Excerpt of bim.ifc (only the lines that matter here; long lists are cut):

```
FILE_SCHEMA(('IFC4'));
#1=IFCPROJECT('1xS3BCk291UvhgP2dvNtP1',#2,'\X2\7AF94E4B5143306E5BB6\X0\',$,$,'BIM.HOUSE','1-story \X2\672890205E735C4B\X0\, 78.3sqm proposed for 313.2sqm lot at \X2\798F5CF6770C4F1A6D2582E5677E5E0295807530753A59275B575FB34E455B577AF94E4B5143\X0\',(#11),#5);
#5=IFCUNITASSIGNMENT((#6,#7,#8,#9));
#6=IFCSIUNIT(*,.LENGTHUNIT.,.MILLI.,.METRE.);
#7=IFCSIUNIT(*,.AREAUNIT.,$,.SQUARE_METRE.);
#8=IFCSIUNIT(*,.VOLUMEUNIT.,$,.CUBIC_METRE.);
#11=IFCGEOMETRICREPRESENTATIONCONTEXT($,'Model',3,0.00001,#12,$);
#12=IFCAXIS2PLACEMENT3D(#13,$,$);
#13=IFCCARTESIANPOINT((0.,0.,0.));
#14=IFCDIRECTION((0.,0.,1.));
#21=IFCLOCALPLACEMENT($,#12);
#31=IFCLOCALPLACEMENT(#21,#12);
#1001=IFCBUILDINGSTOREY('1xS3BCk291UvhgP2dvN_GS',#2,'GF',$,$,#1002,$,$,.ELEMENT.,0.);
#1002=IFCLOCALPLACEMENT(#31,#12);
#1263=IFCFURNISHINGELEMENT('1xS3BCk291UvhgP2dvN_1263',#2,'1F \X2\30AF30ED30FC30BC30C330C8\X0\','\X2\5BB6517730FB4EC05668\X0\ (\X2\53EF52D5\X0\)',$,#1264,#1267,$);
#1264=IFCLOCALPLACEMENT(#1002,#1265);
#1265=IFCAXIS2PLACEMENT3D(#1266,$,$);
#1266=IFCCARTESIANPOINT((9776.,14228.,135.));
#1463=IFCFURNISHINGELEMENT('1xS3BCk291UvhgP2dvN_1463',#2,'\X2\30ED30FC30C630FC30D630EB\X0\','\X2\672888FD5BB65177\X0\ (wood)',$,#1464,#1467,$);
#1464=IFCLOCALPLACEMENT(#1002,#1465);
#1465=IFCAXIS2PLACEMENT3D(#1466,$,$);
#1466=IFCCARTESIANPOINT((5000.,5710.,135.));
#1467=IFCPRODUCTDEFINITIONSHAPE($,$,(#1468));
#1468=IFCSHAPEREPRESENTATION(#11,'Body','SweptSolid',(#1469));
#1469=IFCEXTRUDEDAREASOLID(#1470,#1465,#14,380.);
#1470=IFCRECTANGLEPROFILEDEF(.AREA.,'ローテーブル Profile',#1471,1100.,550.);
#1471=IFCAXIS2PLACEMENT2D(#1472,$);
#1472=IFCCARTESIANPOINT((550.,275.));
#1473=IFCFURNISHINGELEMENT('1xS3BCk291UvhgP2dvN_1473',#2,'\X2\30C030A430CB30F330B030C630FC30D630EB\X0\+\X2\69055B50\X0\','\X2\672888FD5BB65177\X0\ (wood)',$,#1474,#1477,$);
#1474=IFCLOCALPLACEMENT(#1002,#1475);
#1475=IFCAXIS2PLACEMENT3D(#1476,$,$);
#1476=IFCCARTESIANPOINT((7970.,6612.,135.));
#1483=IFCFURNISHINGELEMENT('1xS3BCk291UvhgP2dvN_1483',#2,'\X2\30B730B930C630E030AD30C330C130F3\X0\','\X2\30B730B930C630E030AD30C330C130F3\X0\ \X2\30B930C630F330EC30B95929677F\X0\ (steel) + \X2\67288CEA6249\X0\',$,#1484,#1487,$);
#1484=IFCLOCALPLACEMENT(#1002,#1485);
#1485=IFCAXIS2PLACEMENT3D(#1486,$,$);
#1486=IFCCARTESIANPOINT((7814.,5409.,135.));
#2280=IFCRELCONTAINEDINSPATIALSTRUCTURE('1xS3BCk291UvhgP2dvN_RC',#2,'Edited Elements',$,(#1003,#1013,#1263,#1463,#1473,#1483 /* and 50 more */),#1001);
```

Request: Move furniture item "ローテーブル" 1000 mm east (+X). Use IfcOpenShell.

```python
import ifcopenshell
import ifcopenshell.api.geometry
import ifcopenshell.util.placement

model = ifcopenshell.open("bim.ifc")

item = model.by_guid("1xS3BCk291UvhgP2dvN_1463")
matrix = ifcopenshell.util.placement.get_local_placement(item.ObjectPlacement)
matrix[0, 3] += 1000.0
ifcopenshell.api.geometry.edit_object_placement(model, product=item, matrix=matrix, is_si=False)

print(ifcopenshell.util.placement.get_local_placement(item.ObjectPlacement).round(3) + 0.0)

model.write("bim_updated.ifc")
```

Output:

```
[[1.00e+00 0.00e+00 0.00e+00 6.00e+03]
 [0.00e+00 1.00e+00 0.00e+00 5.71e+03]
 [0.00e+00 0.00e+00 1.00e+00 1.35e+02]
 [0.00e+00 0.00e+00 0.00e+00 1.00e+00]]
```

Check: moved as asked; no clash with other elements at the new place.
